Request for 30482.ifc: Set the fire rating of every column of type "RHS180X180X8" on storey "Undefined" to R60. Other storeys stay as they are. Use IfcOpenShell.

First a look at what the model holds.

```python
import ifcopenshell
import ifcopenshell.util.element

model = ifcopenshell.open("30482.ifc")
print(model.schema)
storey = next(s for s in model.by_type("IfcBuildingStorey") if s.Name == "Undefined")
columns = [e for e in ifcopenshell.util.element.get_decomposition(storey) if e.is_a("IfcColumn")]
seen = {}
for e in columns:
    element_type = ifcopenshell.util.element.get_type(e)
    key = (element_type.Name if element_type != e and element_type else None, ifcopenshell.util.element.get_pset(e, "Pset_ColumnCommon", "FireRating"))
    seen[key] = seen.get(key, 0) + 1
for (name, value), count in sorted(seen.items(), key=str):
    print(count, "x", name, "|", value)
```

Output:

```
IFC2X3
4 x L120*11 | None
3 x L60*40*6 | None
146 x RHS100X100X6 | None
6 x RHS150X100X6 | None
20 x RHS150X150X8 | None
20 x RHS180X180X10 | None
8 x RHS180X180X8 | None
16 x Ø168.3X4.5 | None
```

```python
import ifcopenshell
import ifcopenshell.api.pset
import ifcopenshell.util.element

model = ifcopenshell.open("30482.ifc")

storey = next(s for s in model.by_type("IfcBuildingStorey") if s.Name == "Undefined")
columns = [e for e in ifcopenshell.util.element.get_decomposition(storey) if e.is_a("IfcColumn")]

count = 0
for e in columns:
    element_type = ifcopenshell.util.element.get_type(e)
    if element_type in (None, e) or element_type.Name != "RHS180X180X8":
        continue
    # add_pset returns the element's existing set when there is one.
    pset = ifcopenshell.api.pset.add_pset(model, product=e, name="Pset_ColumnCommon")
    ifcopenshell.api.pset.edit_pset(model, pset=pset, properties={"FireRating": "R60"})
    count += 1

print(count, "columns updated")

model.write("30482_v2.ifc")
```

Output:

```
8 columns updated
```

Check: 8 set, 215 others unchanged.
